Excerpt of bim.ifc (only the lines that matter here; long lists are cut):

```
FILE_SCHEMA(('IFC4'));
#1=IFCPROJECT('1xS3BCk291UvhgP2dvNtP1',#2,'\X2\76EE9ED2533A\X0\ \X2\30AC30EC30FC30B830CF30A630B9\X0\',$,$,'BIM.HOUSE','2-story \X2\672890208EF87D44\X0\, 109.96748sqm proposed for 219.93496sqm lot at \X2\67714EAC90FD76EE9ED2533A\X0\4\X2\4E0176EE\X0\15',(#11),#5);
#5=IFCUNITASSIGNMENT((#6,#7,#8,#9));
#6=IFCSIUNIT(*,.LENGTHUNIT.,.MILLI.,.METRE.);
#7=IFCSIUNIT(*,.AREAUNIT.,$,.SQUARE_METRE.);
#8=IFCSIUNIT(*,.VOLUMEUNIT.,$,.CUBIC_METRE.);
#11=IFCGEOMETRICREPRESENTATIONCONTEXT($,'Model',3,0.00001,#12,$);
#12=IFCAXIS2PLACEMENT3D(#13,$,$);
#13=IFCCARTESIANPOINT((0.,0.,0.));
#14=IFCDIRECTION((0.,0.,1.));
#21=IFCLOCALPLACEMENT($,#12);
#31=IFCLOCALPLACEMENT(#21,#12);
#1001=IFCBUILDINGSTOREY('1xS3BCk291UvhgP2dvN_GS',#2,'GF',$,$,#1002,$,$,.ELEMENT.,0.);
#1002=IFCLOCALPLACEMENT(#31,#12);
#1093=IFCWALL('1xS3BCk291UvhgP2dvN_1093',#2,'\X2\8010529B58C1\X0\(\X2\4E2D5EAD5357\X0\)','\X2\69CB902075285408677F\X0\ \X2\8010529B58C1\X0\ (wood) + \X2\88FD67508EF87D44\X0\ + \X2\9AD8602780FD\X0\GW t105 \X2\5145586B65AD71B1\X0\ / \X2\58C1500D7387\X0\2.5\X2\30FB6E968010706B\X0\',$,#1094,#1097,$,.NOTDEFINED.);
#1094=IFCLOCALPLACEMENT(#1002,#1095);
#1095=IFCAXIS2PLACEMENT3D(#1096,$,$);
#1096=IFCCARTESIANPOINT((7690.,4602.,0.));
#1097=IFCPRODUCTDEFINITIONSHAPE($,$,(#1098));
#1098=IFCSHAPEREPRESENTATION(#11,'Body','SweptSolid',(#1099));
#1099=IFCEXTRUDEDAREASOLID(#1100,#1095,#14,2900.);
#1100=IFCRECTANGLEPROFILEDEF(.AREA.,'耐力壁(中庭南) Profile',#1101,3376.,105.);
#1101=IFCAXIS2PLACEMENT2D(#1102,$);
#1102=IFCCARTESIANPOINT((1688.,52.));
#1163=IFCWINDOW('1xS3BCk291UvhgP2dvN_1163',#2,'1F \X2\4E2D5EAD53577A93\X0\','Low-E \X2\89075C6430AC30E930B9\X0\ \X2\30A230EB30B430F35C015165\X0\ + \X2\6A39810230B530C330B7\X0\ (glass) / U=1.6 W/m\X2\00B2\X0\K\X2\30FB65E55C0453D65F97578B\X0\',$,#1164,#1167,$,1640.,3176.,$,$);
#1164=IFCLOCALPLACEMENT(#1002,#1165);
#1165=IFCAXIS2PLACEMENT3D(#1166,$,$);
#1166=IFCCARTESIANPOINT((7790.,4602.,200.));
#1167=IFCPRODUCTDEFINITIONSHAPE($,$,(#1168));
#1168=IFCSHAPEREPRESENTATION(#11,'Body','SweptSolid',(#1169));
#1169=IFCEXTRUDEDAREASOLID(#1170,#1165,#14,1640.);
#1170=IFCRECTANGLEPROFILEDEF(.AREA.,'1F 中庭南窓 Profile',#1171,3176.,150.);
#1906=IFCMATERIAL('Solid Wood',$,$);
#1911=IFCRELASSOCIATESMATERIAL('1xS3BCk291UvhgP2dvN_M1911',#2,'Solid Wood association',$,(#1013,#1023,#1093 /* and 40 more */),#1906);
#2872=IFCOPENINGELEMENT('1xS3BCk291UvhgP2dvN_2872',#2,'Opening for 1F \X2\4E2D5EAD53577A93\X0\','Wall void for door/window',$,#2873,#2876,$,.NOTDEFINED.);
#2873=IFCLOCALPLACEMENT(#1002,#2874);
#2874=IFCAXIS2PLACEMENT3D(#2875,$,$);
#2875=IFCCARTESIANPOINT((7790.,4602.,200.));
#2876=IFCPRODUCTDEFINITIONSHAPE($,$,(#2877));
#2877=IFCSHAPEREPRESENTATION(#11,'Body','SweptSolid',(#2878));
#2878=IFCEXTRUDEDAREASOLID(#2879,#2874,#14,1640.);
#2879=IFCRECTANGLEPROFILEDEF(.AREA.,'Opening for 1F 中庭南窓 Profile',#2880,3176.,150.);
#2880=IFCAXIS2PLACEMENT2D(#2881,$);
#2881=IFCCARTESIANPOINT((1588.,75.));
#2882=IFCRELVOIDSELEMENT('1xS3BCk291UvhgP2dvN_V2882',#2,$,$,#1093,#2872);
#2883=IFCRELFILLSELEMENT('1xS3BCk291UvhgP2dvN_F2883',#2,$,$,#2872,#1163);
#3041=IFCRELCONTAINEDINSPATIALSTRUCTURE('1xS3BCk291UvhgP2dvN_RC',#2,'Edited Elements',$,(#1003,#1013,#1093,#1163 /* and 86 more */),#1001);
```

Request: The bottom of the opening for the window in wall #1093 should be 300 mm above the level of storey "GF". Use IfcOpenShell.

```python
import numpy as np
import ifcopenshell
import ifcopenshell.api.geometry
import ifcopenshell.geom
import ifcopenshell.util.element
import ifcopenshell.util.placement
import ifcopenshell.util.shape
import ifcopenshell.util.unit

model = ifcopenshell.open("bim.ifc")
unit_scale = ifcopenshell.util.unit.calculate_unit_scale(model)

window = model.by_id(1163)
opening = window.FillsVoids[0].RelatingOpeningElement
storey = ifcopenshell.util.element.get_container(window, ifc_class="IfcBuildingStorey")
level = ifcopenshell.util.placement.get_local_placement(storey.ObjectPlacement)[2, 3]

# The opening's origin need not be at the sill, so measure its lowest point.
shape = ifcopenshell.geom.create_shape(ifcopenshell.geom.settings(), opening)
bottom = ifcopenshell.util.shape.get_shape_bottom_elevation(shape, shape.geometry) / unit_scale
dz = level + 300.0 - bottom

shift = np.array([0.0, 0.0, dz])
# The window is not placed relative to its opening, so move both.
for product in (opening, window):
    matrix = ifcopenshell.util.placement.get_local_placement(product.ObjectPlacement)
    matrix[:3, 3] += shift
    ifcopenshell.api.geometry.edit_object_placement(model, product=product, matrix=matrix, is_si=False)

print(f"moved by {dz * unit_scale:+.3f} m")

model.write("bim_edited.ifc")
```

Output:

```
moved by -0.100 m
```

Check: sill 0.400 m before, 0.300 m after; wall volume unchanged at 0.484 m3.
